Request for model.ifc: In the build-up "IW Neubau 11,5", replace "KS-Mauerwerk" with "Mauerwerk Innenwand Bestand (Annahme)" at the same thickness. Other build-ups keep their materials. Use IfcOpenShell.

First a look at what the model holds.

```python
import ifcopenshell
import ifcopenshell.util.element

model = ifcopenshell.open("model.ifc")
print(model.schema)
for layer_set in model.by_type("IfcMaterialLayerSet"):
    if layer_set.LayerSetName == "IW Neubau 11,5":
        for layer in layer_set.MaterialLayers:
            print(layer.id(), layer.Material and layer.Material.Name, layer.LayerThickness, sep=" | ")
        print(len(ifcopenshell.util.element.get_elements_by_material(model, layer_set)), "elements and types use it")
print(sorted(m.Name for m in model.by_type("IfcMaterial") if m.Name)[:60])
```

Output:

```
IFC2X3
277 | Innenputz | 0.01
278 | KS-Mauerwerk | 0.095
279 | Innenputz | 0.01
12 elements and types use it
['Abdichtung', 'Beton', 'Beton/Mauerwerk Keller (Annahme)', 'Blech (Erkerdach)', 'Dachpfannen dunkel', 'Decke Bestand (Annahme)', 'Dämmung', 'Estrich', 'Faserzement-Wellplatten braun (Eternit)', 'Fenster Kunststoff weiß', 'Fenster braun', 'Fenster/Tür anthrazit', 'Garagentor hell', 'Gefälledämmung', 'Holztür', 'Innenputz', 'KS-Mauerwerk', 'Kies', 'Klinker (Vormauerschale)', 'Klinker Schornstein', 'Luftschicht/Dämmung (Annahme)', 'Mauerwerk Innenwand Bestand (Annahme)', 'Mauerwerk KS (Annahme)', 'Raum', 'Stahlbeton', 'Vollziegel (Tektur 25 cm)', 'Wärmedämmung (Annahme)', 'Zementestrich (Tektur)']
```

```python
import ifcopenshell
import ifcopenshell.api.material

model = ifcopenshell.open("model.ifc")

layer_set = next(s for s in model.by_type("IfcMaterialLayerSet") if s.LayerSetName == "IW Neubau 11,5")
layer = next(l for l in layer_set.MaterialLayers if l.Material and l.Material.Name == "KS-Mauerwerk")
material = next(m for m in model.by_type("IfcMaterial") if m.Name == "Mauerwerk Innenwand Bestand (Annahme)")

# Point this one layer at the other material; renaming the old one would change it everywhere.
ifcopenshell.api.material.edit_layer(model, layer=layer, attributes={}, material=material)

print([l.Material.Name if l.Material else None for l in layer_set.MaterialLayers])

model.write("model_updated.ifc")
```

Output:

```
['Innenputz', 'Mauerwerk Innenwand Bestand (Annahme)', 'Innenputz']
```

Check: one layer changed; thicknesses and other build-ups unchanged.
